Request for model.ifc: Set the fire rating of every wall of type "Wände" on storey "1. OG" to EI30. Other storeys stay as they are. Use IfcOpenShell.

First a look at what the model holds.

```python
import ifcopenshell
import ifcopenshell.util.element

model = ifcopenshell.open("model.ifc")
print(model.schema)
storey = next(s for s in model.by_type("IfcBuildingStorey") if s.Name == "1. OG")
walls = [e for e in ifcopenshell.util.element.get_decomposition(storey) if e.is_a("IfcWall")]
seen = {}
for e in walls:
    element_type = ifcopenshell.util.element.get_type(e)
    key = (element_type.Name if element_type != e and element_type else None, ifcopenshell.util.element.get_pset(e, "Pset_WallCommon", "FireRating"))
    seen[key] = seen.get(key, 0) + 1
for (name, value), count in sorted(seen.items(), key=str):
    print(count, "x", name, "|", value)
```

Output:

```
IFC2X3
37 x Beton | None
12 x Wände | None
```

```python
import ifcopenshell
import ifcopenshell.api.pset
import ifcopenshell.util.element

model = ifcopenshell.open("model.ifc")

storey = next(s for s in model.by_type("IfcBuildingStorey") if s.Name == "1. OG")
walls = [e for e in ifcopenshell.util.element.get_decomposition(storey) if e.is_a("IfcWall")]

count = 0
for e in walls:
    element_type = ifcopenshell.util.element.get_type(e)
    if element_type in (None, e) or element_type.Name != "Wände":
        continue
    # add_pset returns the element's existing set when there is one.
    pset = ifcopenshell.api.pset.add_pset(model, product=e, name="Pset_WallCommon")
    ifcopenshell.api.pset.edit_pset(model, pset=pset, properties={"FireRating": "EI30"})
    count += 1

print(count, "walls updated")

model.write("model_rev.ifc")
```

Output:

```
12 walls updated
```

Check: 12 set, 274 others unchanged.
